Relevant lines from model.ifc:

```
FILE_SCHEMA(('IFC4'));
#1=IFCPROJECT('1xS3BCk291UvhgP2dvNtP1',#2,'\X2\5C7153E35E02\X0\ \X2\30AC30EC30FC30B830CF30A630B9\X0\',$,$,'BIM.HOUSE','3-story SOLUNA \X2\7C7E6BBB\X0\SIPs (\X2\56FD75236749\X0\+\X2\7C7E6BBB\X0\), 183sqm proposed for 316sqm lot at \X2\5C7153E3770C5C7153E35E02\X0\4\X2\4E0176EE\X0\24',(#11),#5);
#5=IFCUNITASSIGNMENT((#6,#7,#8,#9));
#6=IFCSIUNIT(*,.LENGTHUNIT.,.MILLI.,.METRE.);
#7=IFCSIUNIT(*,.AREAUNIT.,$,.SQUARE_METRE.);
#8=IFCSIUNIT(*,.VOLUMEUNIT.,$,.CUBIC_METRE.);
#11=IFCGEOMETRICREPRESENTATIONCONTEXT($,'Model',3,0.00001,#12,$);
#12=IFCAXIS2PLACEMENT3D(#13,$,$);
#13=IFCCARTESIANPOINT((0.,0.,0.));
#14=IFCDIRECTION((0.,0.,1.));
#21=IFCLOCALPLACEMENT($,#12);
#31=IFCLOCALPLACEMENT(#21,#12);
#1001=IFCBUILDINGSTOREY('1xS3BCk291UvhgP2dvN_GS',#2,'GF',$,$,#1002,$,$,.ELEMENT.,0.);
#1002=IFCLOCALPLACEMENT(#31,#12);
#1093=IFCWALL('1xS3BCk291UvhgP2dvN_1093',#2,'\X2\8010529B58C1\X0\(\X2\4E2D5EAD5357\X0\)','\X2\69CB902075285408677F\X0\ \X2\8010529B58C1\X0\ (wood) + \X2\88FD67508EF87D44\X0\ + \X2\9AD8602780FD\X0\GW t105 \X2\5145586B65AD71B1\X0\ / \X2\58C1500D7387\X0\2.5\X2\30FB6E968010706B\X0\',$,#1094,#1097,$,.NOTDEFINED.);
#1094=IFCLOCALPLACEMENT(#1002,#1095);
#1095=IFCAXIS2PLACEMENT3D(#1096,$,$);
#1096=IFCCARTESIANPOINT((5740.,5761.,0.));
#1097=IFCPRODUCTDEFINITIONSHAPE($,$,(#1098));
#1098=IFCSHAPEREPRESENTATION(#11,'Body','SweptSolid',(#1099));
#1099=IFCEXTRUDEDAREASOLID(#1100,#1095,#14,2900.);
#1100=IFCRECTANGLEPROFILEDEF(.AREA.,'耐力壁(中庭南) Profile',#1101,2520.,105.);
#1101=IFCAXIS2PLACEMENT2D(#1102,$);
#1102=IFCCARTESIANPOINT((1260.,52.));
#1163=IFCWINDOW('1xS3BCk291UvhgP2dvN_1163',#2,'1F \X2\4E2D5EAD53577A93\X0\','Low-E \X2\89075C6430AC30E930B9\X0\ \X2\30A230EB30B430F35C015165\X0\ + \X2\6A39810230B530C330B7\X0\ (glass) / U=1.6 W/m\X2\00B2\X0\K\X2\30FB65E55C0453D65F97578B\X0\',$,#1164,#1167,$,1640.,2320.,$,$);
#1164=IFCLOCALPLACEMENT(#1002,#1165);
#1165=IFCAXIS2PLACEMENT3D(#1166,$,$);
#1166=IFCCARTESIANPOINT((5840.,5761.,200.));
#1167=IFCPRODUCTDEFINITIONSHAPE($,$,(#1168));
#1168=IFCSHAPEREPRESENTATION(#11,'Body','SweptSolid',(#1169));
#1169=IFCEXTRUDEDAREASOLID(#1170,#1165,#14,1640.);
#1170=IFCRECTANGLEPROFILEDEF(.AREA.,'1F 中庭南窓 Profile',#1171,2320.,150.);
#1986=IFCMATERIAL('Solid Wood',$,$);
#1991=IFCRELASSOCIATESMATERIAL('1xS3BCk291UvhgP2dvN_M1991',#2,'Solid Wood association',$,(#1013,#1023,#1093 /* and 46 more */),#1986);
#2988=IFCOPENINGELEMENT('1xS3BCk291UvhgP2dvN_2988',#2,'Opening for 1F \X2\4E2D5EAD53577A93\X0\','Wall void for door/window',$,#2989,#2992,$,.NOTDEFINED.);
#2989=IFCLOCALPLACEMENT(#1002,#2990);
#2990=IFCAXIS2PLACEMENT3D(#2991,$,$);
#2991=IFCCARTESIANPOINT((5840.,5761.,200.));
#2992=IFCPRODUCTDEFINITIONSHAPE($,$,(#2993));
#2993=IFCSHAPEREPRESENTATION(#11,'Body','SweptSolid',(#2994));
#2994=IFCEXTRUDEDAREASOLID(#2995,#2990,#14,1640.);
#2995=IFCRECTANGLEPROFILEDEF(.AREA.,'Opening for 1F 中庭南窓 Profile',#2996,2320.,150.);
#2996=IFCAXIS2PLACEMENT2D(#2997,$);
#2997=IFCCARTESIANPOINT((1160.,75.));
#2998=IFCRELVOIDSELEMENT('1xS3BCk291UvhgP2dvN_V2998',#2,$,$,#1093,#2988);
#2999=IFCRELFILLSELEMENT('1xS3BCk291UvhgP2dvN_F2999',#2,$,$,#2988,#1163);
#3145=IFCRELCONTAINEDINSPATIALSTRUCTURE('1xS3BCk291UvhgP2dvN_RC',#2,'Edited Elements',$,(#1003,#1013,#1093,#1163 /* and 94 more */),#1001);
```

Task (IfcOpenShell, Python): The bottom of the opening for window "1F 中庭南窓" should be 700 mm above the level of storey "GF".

```python
import numpy as np
import ifcopenshell
import ifcopenshell.api.geometry
import ifcopenshell.geom
import ifcopenshell.util.element
import ifcopenshell.util.placement
import ifcopenshell.util.shape
import ifcopenshell.util.unit

model = ifcopenshell.open("model.ifc")
unit_scale = ifcopenshell.util.unit.calculate_unit_scale(model)

window = model.by_guid("1xS3BCk291UvhgP2dvN_1163")
opening = window.FillsVoids[0].RelatingOpeningElement
storey = ifcopenshell.util.element.get_container(window, ifc_class="IfcBuildingStorey")
level = ifcopenshell.util.placement.get_local_placement(storey.ObjectPlacement)[2, 3]

# The opening's origin need not be at the sill, so measure its lowest point.
shape = ifcopenshell.geom.create_shape(ifcopenshell.geom.settings(), opening)
bottom = ifcopenshell.util.shape.get_shape_bottom_elevation(shape, shape.geometry) / unit_scale
dz = level + 0.7 / unit_scale - bottom

shift = np.array([0.0, 0.0, dz])
# The window is not placed relative to its opening, so move both.
for product in (opening, window):
    matrix = ifcopenshell.util.placement.get_local_placement(product.ObjectPlacement)
    matrix[:3, 3] += shift
    ifcopenshell.api.geometry.edit_object_placement(model, product=product, matrix=matrix, is_si=False)

print(f"moved by {dz * unit_scale:+.3f} m")

model.write("model_rev.ifc")
```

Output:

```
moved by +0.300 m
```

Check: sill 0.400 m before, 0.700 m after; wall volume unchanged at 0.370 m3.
